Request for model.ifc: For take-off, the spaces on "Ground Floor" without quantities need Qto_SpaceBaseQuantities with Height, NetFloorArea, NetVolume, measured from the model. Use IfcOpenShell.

First a look at what the model holds.

```python
import ifcopenshell
import ifcopenshell.util.element
import ifcopenshell.util.unit

model = ifcopenshell.open("model.ifc")
print(model.schema)
for unit_type in ("LENGTHUNIT", "AREAUNIT", "VOLUMEUNIT"):
    print(unit_type, ifcopenshell.util.unit.calculate_unit_scale(model, unit_type))
storey = next(s for s in model.by_type("IfcBuildingStorey") if s.Name == "Ground Floor")
spaces = [e for e in ifcopenshell.util.element.get_decomposition(storey) if e.is_a("IfcSpace")]
for e in sorted(spaces, key=lambda e: e.id()):
    print(e.id(), e.is_a(), e.Name, list(ifcopenshell.util.element.get_psets(e, qtos_only=True)), sep=" | ")
```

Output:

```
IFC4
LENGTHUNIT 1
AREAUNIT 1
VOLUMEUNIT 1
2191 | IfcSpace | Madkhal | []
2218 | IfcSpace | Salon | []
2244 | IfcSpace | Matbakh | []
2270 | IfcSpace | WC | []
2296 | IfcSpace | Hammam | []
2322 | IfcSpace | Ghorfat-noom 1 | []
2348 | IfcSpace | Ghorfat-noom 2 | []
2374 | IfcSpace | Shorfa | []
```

```python
import ifcopenshell
import ifcopenshell.api.pset
import ifcopenshell.geom
import ifcopenshell.util.element
import ifcopenshell.util.shape
import ifcopenshell.util.unit

model = ifcopenshell.open("model.ifc")
unit_scale = ifcopenshell.util.unit.calculate_unit_scale(model)
area_scale = ifcopenshell.util.unit.calculate_unit_scale(model, "AREAUNIT")
volume_scale = ifcopenshell.util.unit.calculate_unit_scale(model, "VOLUMEUNIT")
settings = ifcopenshell.geom.settings()

storey = next(s for s in model.by_type("IfcBuildingStorey") if s.Name == "Ground Floor")
spaces = [e for e in ifcopenshell.util.element.get_decomposition(storey) if e.is_a("IfcSpace")]

for e in sorted(spaces, key=lambda e: e.id()):
    if ifcopenshell.util.element.get_psets(e, qtos_only=True, should_inherit=False):
        continue
    # Geometry comes back in metres, in the element's own axes.
    shape = ifcopenshell.geom.create_shape(settings, e)
    values = {
        "Height": ifcopenshell.util.shape.get_z(shape.geometry) / unit_scale,
        "NetFloorArea": ifcopenshell.util.shape.get_footprint_area(shape.geometry) / area_scale,
        "NetVolume": ifcopenshell.util.shape.get_volume(shape.geometry) / volume_scale,
    }
    qto = ifcopenshell.api.pset.add_qto(model, product=e, name="Qto_SpaceBaseQuantities")
    ifcopenshell.api.pset.edit_qto(model, qto=qto, properties=values)
    print(e.id(), {k: round(v, 3) for k, v in values.items()})

model.write("model_updated.ifc")
```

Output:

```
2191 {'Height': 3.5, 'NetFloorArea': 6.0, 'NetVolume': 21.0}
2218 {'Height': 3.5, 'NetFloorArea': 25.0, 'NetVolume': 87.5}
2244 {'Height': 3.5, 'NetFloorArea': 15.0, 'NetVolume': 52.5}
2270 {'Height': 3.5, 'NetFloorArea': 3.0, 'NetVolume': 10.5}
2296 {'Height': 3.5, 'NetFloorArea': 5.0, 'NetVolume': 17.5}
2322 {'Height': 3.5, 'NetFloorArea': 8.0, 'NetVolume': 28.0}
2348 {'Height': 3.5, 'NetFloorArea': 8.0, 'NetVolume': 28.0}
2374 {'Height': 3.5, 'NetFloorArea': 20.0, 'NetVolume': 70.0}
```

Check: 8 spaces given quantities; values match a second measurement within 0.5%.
